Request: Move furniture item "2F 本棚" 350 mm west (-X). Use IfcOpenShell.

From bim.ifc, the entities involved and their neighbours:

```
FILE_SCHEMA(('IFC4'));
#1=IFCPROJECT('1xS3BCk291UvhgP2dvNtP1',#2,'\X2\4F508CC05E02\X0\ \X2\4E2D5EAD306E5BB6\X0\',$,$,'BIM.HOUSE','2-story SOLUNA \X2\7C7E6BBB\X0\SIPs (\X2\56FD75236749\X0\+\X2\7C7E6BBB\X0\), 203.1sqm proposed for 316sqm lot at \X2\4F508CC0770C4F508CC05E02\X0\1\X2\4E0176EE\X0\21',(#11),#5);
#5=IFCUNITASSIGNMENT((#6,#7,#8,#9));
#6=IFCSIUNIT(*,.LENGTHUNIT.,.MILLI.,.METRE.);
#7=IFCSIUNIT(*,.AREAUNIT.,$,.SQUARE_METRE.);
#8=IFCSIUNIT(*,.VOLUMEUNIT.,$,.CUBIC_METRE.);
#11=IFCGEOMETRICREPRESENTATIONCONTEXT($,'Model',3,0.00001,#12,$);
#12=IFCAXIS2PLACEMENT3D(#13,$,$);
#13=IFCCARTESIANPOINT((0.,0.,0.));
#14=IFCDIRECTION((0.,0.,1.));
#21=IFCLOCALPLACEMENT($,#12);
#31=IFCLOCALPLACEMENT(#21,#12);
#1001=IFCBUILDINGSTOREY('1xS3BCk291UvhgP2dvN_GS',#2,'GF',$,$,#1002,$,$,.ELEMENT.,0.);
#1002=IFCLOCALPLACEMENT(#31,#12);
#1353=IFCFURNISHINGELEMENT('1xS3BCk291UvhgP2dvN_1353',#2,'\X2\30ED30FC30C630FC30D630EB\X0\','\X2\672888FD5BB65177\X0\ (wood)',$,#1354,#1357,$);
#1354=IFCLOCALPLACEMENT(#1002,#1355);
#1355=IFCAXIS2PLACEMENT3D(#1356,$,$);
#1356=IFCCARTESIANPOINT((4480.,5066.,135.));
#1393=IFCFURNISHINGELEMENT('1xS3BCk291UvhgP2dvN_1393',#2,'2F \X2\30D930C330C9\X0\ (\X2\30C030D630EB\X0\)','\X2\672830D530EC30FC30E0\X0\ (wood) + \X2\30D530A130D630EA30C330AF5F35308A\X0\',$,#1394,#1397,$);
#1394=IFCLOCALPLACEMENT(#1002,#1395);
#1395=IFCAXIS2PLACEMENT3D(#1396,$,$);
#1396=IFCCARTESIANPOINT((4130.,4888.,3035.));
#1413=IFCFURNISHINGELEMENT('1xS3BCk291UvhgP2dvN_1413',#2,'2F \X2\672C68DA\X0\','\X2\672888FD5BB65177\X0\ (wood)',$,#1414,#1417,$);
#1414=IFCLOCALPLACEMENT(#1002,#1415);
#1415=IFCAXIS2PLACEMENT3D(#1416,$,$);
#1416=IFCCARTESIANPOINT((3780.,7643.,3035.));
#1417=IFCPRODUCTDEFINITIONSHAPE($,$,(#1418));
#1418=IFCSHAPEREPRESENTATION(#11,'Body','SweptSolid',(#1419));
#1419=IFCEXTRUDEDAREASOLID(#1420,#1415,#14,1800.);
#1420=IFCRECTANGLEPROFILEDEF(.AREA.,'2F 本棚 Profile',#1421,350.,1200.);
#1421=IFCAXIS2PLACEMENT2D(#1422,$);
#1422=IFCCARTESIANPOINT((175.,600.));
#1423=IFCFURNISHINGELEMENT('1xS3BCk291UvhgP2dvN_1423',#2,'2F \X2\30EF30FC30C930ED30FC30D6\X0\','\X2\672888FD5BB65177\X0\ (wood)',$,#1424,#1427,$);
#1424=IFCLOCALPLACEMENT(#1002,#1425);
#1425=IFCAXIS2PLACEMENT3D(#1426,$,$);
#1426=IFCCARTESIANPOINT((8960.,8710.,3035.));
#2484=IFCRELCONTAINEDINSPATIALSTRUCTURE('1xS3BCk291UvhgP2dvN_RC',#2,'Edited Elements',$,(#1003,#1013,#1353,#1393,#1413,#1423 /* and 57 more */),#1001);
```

```python
import ifcopenshell
import ifcopenshell.api.geometry
import ifcopenshell.util.placement
import ifcopenshell.util.unit

model = ifcopenshell.open("bim.ifc")
unit_scale = ifcopenshell.util.unit.calculate_unit_scale(model)

item = model.by_guid("1xS3BCk291UvhgP2dvN_1413")
matrix = ifcopenshell.util.placement.get_local_placement(item.ObjectPlacement)
matrix[0, 3] -= 0.35 / unit_scale
ifcopenshell.api.geometry.edit_object_placement(model, product=item, matrix=matrix, is_si=False)

print(ifcopenshell.util.placement.get_local_placement(item.ObjectPlacement).round(3) + 0.0)

model.write("bim_rev.ifc")
```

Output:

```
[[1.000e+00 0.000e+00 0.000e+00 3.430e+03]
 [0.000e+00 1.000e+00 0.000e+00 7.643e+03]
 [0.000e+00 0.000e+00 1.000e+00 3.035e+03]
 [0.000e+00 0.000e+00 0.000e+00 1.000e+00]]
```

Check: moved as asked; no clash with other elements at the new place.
